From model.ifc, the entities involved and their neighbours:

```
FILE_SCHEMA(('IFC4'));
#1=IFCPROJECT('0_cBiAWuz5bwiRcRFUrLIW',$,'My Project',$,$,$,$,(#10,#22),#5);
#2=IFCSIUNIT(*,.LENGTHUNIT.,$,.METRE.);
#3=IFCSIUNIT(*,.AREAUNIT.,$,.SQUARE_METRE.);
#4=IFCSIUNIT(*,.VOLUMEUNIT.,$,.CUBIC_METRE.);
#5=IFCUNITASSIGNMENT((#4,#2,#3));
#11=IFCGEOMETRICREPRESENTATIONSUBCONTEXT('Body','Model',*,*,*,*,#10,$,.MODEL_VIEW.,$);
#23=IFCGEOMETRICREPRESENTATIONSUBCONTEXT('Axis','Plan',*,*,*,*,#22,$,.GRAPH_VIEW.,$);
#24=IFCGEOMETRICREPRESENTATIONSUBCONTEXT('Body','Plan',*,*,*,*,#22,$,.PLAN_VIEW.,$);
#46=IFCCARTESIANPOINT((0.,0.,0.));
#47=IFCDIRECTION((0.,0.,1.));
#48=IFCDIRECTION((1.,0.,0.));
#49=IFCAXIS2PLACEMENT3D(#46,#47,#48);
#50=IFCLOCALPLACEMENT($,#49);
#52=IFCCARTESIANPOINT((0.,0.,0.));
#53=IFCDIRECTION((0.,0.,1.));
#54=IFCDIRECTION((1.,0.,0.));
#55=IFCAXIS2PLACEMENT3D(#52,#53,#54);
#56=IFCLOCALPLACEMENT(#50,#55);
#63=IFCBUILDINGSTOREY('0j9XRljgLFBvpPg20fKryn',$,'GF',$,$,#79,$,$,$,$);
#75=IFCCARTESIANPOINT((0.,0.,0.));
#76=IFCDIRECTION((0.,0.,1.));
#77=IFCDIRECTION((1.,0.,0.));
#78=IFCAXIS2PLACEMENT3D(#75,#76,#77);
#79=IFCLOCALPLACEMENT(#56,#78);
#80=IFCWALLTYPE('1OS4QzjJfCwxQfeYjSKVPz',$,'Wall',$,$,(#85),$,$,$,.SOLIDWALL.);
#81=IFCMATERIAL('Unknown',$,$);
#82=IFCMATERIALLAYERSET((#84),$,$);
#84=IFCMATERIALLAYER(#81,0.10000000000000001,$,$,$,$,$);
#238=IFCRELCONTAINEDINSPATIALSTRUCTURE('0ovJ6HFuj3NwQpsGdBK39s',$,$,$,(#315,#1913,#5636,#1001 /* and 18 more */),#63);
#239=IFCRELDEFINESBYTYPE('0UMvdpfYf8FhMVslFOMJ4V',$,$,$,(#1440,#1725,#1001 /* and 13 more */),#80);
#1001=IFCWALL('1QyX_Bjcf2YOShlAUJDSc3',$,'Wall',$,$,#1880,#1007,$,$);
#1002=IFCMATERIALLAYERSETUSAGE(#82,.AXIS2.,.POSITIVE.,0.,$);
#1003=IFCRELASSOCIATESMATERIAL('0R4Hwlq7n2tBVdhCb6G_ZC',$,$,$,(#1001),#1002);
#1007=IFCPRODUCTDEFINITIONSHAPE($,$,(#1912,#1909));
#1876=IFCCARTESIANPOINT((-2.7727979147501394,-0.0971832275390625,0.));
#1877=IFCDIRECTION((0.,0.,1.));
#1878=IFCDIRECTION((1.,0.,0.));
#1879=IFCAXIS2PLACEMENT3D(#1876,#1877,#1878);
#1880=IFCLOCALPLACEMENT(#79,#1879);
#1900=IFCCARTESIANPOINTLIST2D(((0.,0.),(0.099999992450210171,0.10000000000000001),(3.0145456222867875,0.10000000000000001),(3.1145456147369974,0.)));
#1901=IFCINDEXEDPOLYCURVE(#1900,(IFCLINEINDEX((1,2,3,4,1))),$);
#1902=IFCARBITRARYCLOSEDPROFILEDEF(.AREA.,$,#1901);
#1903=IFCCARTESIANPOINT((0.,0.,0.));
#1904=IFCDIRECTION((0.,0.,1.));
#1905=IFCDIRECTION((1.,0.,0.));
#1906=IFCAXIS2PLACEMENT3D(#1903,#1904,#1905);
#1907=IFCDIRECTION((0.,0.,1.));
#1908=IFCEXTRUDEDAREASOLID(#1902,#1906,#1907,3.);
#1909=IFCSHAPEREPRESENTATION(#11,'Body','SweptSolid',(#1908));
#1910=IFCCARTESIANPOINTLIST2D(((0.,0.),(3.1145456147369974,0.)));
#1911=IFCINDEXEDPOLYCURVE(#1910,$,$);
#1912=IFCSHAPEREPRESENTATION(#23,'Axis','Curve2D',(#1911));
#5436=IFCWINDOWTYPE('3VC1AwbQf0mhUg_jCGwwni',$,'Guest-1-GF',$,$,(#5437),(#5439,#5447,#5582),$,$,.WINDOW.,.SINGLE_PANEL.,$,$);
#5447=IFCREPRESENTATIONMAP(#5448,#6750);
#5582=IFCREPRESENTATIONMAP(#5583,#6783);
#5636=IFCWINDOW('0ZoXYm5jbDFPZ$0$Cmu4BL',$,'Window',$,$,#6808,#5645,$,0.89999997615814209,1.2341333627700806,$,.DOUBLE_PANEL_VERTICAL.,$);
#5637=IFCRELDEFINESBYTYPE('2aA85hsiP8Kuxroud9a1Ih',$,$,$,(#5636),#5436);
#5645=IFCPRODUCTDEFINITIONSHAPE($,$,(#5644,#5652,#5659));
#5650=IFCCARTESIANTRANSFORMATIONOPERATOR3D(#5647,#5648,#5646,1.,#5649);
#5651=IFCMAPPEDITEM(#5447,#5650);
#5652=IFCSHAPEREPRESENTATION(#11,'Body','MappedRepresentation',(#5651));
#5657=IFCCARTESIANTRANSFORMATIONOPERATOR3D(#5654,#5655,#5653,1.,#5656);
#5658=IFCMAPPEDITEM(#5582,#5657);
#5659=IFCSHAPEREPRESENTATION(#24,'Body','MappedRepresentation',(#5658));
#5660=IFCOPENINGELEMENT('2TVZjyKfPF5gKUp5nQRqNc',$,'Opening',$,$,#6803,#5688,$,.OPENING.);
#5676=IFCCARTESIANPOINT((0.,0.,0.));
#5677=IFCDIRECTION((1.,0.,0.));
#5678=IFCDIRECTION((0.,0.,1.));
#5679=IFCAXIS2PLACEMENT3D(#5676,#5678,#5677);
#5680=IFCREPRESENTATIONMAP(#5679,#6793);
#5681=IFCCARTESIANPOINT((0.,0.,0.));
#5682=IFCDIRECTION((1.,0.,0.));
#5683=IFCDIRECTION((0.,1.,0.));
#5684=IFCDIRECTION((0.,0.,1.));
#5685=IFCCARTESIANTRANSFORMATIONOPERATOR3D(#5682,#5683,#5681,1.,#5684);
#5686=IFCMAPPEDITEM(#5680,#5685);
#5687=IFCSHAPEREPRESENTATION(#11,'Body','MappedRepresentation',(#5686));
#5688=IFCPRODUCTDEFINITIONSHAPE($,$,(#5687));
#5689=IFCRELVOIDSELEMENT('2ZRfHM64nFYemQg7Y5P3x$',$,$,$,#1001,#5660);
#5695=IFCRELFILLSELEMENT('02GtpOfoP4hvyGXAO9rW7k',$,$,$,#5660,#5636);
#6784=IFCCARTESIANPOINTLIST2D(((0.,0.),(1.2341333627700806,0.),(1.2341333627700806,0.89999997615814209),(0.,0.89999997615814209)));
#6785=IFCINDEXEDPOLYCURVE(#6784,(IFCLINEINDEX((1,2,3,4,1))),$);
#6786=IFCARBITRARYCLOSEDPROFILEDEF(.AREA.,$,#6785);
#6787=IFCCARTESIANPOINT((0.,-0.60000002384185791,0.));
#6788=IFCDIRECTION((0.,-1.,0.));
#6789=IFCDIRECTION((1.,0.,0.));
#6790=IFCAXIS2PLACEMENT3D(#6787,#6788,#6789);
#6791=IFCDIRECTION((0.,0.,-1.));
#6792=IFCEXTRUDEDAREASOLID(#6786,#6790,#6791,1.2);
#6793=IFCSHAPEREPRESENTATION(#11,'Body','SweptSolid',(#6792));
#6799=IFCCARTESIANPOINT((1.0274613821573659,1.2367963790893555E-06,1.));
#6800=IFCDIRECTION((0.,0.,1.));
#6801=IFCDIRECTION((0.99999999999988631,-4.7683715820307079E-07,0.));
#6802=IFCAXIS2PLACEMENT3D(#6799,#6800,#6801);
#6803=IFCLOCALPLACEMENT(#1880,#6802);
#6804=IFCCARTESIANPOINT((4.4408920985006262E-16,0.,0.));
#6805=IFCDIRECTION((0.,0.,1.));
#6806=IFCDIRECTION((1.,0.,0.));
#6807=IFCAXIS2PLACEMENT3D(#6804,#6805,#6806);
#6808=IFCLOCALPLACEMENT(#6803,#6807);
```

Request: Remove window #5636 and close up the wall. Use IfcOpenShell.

```python
import ifcopenshell
import ifcopenshell.api.feature
import ifcopenshell.api.root
import ifcopenshell.geom
import ifcopenshell.util.shape

model = ifcopenshell.open("model.ifc")
settings = ifcopenshell.geom.settings()


def volume(element):
    """Net volume in cubic metres, openings subtracted."""
    shape = ifcopenshell.geom.create_shape(settings, element)
    return ifcopenshell.util.shape.get_volume(shape.geometry)


window = model.by_guid("0ZoXYm5jbDFPZ$0$Cmu4BL")
opening = window.FillsVoids[0].RelatingOpeningElement
wall = opening.VoidsElements[0].RelatingBuildingElement
before = volume(wall)

ifcopenshell.api.root.remove_product(model, product=window)
ifcopenshell.api.feature.remove_feature(model, feature=opening)

after = volume(wall)

print(f"wall volume {before:.3f} -> {after:.3f} m3")

model.write("model_rev.ifc")
```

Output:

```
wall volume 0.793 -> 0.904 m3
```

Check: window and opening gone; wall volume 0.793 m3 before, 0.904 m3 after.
